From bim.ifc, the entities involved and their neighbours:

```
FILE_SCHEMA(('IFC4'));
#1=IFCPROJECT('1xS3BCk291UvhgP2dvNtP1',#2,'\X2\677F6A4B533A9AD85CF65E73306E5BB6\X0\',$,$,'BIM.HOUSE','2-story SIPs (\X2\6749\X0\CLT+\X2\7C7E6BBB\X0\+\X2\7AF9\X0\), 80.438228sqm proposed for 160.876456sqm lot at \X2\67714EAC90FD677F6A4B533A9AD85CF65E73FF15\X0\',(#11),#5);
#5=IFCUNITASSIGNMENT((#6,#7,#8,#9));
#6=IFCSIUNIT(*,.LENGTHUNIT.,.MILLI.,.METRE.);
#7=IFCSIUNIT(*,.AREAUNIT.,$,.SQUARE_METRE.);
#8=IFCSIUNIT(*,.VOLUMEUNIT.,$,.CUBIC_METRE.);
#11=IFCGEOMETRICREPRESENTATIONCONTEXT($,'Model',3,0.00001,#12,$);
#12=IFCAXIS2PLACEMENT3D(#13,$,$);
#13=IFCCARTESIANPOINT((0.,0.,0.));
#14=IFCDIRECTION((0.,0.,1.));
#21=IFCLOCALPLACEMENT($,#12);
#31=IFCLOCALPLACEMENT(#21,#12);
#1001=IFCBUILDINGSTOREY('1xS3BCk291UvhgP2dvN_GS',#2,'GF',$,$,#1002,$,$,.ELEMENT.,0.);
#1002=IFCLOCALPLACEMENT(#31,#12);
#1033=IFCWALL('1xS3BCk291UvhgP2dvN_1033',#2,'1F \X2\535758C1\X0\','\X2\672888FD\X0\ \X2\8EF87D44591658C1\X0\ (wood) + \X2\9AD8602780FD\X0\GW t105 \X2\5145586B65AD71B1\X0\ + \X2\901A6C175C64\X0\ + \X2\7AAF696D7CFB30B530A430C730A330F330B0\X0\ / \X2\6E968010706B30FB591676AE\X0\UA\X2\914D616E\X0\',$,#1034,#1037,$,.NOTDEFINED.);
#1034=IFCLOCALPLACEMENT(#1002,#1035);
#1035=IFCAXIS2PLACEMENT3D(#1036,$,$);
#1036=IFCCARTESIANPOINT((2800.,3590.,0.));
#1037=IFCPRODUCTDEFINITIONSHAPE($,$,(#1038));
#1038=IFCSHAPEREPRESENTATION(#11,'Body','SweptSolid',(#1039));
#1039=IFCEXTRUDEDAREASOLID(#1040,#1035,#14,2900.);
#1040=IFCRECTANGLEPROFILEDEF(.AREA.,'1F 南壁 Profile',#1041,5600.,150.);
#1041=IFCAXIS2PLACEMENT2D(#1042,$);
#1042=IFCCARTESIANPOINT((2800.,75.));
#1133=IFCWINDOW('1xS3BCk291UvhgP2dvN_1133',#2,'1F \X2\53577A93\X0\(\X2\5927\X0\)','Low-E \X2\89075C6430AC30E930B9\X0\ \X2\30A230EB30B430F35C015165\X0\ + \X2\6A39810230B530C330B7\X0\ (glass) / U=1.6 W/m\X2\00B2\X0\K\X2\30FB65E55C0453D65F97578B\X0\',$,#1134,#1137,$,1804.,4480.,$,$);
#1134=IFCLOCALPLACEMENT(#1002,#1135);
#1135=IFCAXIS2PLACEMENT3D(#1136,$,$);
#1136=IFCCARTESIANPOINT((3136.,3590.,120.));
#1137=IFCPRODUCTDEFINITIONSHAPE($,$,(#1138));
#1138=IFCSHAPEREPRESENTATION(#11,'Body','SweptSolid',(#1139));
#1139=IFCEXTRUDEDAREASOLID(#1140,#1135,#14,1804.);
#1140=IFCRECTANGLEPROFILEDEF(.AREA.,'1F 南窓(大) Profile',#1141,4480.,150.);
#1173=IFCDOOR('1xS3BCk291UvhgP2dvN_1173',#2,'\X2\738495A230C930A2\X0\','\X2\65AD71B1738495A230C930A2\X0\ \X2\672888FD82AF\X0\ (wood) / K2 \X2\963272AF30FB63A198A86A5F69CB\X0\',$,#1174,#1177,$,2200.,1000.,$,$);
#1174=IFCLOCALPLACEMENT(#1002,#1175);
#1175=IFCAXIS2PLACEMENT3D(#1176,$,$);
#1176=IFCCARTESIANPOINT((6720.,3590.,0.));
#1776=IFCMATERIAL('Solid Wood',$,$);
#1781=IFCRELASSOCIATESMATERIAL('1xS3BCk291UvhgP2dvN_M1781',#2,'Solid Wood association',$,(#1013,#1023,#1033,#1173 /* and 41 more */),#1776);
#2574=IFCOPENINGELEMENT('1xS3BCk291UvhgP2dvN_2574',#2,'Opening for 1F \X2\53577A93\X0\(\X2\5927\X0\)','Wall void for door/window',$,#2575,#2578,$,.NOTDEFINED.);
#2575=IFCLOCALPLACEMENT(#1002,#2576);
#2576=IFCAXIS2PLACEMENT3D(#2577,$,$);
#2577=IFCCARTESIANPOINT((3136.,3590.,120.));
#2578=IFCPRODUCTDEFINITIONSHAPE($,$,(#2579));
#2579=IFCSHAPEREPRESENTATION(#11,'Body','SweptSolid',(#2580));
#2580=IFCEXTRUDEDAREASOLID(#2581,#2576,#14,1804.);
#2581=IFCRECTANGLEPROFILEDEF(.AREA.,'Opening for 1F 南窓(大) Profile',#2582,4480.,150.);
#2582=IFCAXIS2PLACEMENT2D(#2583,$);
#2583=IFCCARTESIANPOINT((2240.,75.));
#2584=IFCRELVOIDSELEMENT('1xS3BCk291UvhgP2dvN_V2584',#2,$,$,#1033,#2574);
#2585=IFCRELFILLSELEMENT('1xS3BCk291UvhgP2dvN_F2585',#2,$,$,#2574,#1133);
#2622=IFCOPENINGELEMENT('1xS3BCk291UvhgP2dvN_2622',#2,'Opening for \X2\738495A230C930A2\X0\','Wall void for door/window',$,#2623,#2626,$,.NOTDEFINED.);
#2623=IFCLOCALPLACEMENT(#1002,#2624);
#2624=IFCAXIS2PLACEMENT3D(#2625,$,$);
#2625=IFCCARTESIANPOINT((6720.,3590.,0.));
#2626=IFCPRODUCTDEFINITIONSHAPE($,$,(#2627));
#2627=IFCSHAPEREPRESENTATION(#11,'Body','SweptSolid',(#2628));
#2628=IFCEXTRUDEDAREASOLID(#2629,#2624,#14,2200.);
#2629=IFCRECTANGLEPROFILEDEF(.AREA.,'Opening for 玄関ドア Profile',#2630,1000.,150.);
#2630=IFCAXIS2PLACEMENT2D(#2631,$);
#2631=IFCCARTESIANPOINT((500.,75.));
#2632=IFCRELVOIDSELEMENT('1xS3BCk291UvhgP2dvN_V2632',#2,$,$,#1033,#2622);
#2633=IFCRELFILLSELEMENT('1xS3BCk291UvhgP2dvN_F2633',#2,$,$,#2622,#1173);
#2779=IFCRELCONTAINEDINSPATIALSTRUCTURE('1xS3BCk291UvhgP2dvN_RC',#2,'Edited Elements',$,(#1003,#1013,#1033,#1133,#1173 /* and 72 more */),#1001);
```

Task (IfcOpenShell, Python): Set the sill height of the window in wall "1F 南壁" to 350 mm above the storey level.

```python
import numpy as np
import ifcopenshell
import ifcopenshell.api.geometry
import ifcopenshell.geom
import ifcopenshell.util.element
import ifcopenshell.util.placement
import ifcopenshell.util.shape
import ifcopenshell.util.unit

model = ifcopenshell.open("bim.ifc")
unit_scale = ifcopenshell.util.unit.calculate_unit_scale(model)

window = model.by_guid("1xS3BCk291UvhgP2dvN_1133")
opening = window.FillsVoids[0].RelatingOpeningElement
storey = ifcopenshell.util.element.get_container(window, ifc_class="IfcBuildingStorey")
level = ifcopenshell.util.placement.get_local_placement(storey.ObjectPlacement)[2, 3]

# The opening's origin need not be at the sill, so measure its lowest point.
shape = ifcopenshell.geom.create_shape(ifcopenshell.geom.settings(), opening)
bottom = ifcopenshell.util.shape.get_shape_bottom_elevation(shape, shape.geometry) / unit_scale
dz = level + 0.35 / unit_scale - bottom

shift = np.array([0.0, 0.0, dz])
# The window is not placed relative to its opening, so move both.
for product in (opening, window):
    matrix = ifcopenshell.util.placement.get_local_placement(product.ObjectPlacement)
    matrix[:3, 3] += shift
    ifcopenshell.api.geometry.edit_object_placement(model, product=product, matrix=matrix, is_si=False)

print(f"moved by {dz * unit_scale:+.3f} m")

model.write("bim_edited.ifc")
```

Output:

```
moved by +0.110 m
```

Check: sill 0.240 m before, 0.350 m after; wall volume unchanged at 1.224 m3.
